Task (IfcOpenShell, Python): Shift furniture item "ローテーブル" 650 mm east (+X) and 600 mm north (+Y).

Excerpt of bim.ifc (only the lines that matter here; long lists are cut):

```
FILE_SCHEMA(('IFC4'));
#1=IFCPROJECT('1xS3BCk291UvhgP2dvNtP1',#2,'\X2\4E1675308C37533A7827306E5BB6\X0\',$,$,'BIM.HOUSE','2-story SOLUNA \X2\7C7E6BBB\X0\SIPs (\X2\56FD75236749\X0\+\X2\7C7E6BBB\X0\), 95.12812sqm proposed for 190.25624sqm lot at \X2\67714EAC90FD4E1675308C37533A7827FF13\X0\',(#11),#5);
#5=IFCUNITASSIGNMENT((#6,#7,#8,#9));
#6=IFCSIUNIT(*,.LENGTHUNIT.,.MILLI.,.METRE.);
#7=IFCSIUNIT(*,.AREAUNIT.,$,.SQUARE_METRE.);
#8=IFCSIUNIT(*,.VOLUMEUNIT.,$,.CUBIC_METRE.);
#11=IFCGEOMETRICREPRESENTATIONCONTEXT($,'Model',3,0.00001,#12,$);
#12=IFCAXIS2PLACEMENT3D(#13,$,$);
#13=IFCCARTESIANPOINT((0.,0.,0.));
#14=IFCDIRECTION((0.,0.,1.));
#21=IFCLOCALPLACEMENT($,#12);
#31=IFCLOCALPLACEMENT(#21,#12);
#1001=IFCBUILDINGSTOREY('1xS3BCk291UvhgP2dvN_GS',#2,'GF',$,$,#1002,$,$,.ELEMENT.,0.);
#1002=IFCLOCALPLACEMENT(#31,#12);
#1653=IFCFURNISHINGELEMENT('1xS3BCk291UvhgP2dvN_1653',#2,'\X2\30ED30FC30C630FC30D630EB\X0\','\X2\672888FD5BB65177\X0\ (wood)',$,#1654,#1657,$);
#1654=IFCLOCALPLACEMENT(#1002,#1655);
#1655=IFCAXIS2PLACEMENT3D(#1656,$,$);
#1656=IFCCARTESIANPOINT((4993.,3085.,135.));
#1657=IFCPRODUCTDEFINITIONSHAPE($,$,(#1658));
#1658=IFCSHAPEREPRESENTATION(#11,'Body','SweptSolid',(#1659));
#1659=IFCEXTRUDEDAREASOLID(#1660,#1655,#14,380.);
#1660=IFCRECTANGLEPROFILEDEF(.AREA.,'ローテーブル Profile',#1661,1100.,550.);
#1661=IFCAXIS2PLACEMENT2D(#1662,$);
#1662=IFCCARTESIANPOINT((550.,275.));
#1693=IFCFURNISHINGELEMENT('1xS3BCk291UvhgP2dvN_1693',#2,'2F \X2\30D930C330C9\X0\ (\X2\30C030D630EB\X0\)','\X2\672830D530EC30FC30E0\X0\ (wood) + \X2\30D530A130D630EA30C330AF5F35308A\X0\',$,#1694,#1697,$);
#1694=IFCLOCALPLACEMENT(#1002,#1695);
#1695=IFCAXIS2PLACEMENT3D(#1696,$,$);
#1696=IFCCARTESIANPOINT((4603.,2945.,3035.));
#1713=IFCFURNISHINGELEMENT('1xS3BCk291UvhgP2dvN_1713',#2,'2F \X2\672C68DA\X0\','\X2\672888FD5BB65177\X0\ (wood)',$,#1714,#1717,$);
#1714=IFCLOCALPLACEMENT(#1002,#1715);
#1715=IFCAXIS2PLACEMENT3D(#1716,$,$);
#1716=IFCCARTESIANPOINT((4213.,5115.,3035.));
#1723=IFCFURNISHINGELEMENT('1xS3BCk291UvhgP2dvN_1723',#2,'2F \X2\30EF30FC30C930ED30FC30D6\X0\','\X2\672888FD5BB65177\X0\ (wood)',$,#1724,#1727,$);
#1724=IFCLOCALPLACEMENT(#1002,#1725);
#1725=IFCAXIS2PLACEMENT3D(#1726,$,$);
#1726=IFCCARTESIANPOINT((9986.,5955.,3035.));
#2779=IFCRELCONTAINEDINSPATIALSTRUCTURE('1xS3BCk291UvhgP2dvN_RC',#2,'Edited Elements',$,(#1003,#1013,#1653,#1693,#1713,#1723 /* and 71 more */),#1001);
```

```python
import ifcopenshell
import ifcopenshell.api.geometry
import ifcopenshell.util.placement

model = ifcopenshell.open("bim.ifc")

item = model.by_guid("1xS3BCk291UvhgP2dvN_1653")
matrix = ifcopenshell.util.placement.get_local_placement(item.ObjectPlacement)
matrix[0, 3] += 650.0
matrix[1, 3] += 600.0
ifcopenshell.api.geometry.edit_object_placement(model, product=item, matrix=matrix, is_si=False)

print(ifcopenshell.util.placement.get_local_placement(item.ObjectPlacement).round(3) + 0.0)

model.write("bim_rev.ifc")
```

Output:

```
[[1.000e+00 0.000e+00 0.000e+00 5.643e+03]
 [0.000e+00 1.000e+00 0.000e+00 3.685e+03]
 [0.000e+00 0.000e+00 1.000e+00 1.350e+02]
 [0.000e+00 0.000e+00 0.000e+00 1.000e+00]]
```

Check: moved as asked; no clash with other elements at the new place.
